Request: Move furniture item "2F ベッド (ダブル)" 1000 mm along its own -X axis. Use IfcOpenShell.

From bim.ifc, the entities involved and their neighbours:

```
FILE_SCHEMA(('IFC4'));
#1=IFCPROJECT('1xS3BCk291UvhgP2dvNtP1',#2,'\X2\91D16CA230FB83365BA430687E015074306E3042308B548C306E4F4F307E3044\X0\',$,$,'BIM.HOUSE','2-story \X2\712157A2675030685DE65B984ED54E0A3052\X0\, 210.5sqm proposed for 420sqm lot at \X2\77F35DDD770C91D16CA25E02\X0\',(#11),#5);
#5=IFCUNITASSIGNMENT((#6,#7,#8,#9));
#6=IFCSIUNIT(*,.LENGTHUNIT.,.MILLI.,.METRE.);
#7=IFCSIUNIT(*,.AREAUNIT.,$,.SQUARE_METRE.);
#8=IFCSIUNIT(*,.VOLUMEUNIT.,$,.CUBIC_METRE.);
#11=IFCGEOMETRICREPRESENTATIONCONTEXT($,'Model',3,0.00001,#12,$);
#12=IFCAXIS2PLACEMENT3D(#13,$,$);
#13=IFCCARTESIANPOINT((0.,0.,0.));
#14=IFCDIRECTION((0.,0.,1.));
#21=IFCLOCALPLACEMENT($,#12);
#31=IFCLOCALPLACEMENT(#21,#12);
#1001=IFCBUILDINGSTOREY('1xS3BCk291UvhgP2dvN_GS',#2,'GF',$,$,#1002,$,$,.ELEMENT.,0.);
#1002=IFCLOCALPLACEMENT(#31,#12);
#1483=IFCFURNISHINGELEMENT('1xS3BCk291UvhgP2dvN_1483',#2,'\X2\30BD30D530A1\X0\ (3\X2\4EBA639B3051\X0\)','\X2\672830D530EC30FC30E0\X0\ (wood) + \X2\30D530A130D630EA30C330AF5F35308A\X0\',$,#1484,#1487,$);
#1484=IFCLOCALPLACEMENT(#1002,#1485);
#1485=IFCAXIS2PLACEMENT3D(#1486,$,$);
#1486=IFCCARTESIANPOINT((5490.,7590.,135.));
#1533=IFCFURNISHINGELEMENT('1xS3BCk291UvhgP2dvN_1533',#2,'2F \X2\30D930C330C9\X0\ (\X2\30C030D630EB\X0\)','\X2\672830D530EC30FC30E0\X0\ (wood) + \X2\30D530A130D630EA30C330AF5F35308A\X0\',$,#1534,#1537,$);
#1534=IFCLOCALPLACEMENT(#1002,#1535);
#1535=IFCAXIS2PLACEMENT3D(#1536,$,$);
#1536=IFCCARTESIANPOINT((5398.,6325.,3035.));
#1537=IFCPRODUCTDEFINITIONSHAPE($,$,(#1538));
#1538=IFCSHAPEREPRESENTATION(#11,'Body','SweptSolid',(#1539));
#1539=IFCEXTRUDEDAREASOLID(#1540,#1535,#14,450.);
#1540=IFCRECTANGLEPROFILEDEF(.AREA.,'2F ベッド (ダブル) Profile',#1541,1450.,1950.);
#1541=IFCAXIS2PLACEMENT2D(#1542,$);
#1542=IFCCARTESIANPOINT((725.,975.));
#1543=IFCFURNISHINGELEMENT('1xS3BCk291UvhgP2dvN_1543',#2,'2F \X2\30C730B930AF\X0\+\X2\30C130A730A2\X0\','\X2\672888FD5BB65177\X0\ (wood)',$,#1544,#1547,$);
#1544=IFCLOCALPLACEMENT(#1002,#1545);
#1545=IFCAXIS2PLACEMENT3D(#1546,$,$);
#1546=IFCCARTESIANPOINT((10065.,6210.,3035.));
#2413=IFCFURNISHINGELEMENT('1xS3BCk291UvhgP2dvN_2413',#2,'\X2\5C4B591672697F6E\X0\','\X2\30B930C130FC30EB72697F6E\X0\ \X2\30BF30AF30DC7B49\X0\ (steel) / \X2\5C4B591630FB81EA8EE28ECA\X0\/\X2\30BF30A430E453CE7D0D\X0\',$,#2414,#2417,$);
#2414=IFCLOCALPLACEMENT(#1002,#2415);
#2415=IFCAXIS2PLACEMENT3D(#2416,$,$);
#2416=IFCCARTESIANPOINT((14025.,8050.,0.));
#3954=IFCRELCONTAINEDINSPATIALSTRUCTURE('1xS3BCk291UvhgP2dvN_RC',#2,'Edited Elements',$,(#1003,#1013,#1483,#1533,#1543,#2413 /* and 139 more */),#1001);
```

```python
import ifcopenshell
import ifcopenshell.api.geometry
import ifcopenshell.util.placement
import ifcopenshell.util.unit

model = ifcopenshell.open("bim.ifc")
unit_scale = ifcopenshell.util.unit.calculate_unit_scale(model)

item = model.by_guid("1xS3BCk291UvhgP2dvN_1533")
matrix = ifcopenshell.util.placement.get_local_placement(item.ObjectPlacement)
matrix[:3, 3] -= matrix[:3, 0] * 1 / unit_scale
ifcopenshell.api.geometry.edit_object_placement(model, product=item, matrix=matrix, is_si=False)

print(ifcopenshell.util.placement.get_local_placement(item.ObjectPlacement).round(3) + 0.0)

model.write("bim-out.ifc")
```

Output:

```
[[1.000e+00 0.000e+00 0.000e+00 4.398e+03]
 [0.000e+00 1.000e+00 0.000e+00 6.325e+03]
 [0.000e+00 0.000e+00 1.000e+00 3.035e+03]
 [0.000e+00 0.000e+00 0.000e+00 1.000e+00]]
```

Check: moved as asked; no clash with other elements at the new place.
